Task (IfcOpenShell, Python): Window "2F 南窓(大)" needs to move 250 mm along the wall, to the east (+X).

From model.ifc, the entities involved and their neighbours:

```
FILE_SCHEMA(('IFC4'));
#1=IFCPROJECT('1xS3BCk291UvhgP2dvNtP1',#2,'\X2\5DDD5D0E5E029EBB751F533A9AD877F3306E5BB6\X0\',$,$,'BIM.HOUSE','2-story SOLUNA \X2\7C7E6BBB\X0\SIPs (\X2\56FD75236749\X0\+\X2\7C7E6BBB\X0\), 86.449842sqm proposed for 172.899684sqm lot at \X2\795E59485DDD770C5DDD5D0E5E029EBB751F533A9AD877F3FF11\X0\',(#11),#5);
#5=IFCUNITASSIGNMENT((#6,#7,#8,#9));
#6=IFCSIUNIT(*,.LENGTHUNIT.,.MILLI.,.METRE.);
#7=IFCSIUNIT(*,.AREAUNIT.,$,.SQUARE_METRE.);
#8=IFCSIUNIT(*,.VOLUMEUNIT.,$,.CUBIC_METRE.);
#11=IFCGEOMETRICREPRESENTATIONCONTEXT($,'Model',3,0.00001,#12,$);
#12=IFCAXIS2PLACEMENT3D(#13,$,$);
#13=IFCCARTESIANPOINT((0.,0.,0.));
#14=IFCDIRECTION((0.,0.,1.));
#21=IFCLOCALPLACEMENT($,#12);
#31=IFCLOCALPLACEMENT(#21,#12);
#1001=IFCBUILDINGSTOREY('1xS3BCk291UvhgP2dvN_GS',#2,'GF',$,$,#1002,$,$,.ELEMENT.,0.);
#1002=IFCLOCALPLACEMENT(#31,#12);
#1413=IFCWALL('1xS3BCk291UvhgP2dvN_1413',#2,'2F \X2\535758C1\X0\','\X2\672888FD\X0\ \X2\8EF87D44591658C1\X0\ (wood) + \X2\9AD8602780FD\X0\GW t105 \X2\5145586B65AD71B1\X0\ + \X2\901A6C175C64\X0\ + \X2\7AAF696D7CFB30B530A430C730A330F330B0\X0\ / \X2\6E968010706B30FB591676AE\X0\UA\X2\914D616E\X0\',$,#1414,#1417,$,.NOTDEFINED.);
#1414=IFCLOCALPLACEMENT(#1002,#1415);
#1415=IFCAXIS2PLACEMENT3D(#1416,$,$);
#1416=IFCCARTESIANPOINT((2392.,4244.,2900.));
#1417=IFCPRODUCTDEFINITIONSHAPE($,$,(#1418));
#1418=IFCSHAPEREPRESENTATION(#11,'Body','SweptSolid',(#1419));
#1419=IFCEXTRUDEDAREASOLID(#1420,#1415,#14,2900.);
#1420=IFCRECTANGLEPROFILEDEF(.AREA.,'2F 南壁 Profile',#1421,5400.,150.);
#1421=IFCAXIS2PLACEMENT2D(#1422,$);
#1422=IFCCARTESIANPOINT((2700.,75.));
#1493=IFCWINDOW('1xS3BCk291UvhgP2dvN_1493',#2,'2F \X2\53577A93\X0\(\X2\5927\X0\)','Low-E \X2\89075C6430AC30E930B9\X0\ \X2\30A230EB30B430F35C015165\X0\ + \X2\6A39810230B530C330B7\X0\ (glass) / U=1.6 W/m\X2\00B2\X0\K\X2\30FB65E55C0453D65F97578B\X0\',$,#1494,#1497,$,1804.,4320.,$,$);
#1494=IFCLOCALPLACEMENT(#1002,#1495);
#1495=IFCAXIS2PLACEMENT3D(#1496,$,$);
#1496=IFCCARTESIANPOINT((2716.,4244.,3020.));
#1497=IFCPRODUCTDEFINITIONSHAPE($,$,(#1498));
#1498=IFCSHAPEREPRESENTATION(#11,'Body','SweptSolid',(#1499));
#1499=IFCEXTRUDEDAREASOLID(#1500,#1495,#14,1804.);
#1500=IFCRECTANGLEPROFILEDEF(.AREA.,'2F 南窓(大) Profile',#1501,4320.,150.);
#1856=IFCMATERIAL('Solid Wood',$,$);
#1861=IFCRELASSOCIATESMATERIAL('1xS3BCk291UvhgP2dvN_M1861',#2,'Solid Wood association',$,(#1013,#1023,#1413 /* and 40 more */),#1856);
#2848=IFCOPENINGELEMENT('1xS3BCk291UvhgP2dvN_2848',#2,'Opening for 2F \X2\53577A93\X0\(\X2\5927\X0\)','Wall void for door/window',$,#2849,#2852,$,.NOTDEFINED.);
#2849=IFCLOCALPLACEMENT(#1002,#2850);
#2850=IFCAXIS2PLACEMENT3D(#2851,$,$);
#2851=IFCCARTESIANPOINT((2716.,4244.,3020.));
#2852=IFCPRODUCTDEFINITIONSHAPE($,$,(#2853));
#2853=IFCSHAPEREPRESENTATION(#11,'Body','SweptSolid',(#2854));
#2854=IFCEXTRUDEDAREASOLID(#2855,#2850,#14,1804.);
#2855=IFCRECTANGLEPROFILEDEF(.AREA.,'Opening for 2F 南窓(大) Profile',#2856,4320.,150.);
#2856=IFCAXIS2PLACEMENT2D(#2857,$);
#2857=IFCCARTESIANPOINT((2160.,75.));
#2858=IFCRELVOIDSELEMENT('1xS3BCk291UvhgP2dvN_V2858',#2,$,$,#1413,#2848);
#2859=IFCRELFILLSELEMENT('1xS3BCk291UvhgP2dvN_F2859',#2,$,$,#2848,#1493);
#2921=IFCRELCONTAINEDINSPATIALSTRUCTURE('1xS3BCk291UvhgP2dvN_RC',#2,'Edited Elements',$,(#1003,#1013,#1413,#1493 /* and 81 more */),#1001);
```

```python
import ifcopenshell
import ifcopenshell.api.geometry
import ifcopenshell.util.placement

model = ifcopenshell.open("model.ifc")

window = model.by_guid("1xS3BCk291UvhgP2dvN_1493")
opening = window.FillsVoids[0].RelatingOpeningElement
wall = opening.VoidsElements[0].RelatingBuildingElement

wall_matrix = ifcopenshell.util.placement.get_local_placement(wall.ObjectPlacement)
shift = wall_matrix[:3, 0] * 250.0
before = ifcopenshell.util.placement.get_local_placement(window.ObjectPlacement)[:3, 3].copy()

# The window is not placed relative to its opening, so move both.
for product in (opening, window):
    matrix = ifcopenshell.util.placement.get_local_placement(product.ObjectPlacement)
    matrix[:3, 3] += shift
    ifcopenshell.api.geometry.edit_object_placement(model, product=product, matrix=matrix, is_si=False)

after = ifcopenshell.util.placement.get_local_placement(window.ObjectPlacement)[:3, 3]
print("window moved by", (after - before).round(3) + 0.0)

model.write("model_v2.ifc")
```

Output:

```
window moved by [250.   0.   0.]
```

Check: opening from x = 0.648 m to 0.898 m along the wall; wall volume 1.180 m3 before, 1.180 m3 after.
